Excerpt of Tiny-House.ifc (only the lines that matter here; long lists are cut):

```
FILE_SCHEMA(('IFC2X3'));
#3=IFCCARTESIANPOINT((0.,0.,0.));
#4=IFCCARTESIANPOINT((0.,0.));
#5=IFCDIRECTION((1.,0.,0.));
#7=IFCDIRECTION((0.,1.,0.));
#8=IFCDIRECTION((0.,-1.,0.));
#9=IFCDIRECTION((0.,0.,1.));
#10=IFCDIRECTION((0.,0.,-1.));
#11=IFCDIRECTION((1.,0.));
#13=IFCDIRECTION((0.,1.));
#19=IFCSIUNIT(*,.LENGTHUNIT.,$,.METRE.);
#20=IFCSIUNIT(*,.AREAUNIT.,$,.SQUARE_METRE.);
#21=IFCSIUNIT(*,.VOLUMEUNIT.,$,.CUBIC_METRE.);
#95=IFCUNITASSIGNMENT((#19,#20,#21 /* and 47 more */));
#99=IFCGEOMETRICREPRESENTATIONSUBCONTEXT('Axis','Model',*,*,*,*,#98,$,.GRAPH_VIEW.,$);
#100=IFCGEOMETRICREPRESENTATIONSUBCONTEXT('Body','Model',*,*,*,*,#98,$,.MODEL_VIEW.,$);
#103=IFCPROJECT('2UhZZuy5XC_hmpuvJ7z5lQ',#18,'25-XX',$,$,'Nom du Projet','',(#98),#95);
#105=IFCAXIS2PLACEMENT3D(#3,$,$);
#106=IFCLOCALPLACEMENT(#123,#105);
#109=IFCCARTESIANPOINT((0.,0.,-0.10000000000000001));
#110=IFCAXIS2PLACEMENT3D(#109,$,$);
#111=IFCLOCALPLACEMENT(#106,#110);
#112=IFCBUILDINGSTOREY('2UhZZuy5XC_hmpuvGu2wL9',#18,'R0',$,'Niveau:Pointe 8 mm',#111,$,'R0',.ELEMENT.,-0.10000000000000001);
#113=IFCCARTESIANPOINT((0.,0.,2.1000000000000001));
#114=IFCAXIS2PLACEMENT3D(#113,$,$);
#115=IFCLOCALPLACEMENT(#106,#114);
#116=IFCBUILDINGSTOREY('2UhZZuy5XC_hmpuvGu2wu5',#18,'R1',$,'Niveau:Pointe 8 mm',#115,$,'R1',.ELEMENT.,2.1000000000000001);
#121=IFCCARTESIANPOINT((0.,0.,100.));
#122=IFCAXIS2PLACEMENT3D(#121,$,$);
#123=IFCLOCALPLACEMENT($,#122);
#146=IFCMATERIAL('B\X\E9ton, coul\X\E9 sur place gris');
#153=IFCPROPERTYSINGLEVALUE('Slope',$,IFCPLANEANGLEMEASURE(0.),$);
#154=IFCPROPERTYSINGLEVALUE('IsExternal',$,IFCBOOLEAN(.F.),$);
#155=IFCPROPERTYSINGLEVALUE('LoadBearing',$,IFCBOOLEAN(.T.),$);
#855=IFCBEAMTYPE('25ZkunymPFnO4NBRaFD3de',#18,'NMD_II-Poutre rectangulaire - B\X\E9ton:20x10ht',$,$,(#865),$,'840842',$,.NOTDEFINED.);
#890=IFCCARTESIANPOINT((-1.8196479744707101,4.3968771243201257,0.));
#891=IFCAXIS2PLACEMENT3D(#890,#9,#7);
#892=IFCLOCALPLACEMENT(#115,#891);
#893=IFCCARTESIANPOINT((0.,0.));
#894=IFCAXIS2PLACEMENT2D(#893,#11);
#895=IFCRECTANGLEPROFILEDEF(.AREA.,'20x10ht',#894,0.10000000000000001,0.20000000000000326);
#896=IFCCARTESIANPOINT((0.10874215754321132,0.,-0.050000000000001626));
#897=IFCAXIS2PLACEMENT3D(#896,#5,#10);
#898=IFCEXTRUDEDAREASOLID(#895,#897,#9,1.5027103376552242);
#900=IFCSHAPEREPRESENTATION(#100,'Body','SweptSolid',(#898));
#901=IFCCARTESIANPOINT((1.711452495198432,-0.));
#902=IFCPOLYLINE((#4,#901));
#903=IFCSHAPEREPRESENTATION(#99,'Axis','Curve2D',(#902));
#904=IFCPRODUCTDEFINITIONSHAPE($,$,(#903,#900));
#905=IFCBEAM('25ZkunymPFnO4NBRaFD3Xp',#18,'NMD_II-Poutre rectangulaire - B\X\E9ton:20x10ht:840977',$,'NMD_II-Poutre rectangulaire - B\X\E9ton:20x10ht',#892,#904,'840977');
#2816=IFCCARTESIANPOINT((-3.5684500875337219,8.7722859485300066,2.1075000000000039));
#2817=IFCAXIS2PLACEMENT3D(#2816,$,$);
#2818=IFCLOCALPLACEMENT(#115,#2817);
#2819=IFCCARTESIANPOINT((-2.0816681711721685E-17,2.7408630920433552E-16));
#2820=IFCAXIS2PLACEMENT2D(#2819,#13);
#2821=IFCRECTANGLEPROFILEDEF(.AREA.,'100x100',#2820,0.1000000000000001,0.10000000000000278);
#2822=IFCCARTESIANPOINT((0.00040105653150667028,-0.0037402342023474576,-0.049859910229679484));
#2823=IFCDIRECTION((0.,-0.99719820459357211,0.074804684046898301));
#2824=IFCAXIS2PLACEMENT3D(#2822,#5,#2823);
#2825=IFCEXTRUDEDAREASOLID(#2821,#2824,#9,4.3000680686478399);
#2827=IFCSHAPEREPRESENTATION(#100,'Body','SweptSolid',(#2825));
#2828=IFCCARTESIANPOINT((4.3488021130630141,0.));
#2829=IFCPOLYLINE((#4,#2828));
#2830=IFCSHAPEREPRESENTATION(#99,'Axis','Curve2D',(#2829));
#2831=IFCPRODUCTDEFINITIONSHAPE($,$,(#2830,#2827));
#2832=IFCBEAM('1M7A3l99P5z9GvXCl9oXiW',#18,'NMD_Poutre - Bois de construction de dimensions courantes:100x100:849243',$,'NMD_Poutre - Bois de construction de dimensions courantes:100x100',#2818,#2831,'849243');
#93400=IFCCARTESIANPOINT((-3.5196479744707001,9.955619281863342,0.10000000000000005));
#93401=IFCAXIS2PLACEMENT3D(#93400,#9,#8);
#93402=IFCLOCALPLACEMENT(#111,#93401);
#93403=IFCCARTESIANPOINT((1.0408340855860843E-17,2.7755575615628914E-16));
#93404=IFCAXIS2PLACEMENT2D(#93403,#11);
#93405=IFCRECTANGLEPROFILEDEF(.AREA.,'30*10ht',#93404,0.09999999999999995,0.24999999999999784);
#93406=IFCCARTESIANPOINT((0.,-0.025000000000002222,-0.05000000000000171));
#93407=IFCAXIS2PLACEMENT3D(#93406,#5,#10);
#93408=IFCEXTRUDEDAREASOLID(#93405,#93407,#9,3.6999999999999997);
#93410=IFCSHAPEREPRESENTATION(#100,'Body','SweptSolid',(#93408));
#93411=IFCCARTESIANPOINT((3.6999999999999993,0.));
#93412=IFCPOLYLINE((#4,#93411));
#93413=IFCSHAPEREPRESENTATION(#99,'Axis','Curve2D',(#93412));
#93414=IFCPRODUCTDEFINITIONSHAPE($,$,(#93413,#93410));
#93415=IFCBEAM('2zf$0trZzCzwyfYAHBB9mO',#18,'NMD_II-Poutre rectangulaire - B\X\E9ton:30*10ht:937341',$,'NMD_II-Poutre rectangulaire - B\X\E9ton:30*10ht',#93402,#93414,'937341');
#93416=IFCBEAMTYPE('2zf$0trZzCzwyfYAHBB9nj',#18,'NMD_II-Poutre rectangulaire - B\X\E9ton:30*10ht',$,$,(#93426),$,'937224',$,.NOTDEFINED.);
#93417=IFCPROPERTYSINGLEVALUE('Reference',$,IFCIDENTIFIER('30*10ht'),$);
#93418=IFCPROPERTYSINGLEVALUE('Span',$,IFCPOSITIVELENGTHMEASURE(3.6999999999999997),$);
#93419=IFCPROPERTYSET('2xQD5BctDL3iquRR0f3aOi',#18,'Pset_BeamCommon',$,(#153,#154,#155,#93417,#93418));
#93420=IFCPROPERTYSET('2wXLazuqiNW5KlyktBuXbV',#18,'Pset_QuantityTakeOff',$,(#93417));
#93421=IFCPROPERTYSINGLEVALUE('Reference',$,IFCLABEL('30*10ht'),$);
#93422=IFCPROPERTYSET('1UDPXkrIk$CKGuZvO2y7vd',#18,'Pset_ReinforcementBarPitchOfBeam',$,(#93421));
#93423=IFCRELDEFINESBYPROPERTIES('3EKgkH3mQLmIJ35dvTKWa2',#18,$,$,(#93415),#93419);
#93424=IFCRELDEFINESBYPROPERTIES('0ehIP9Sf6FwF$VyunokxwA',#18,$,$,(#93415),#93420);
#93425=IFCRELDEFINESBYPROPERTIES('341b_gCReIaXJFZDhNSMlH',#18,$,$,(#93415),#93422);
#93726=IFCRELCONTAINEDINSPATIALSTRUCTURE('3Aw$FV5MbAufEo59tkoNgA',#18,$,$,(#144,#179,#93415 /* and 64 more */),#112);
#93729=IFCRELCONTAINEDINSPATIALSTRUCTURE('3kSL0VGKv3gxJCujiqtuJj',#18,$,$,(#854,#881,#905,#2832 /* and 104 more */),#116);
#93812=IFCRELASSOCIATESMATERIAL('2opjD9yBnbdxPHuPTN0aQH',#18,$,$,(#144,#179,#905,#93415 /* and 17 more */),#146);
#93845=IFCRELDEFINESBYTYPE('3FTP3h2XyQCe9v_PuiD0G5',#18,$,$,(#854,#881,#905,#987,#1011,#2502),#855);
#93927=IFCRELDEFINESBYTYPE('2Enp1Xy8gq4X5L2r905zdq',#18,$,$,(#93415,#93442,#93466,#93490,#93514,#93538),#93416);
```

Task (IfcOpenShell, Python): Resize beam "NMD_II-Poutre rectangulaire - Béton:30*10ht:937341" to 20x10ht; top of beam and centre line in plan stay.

```python
import ifcopenshell
import ifcopenshell.api.pset
import ifcopenshell.api.type
import ifcopenshell.util.element
import ifcopenshell.util.representation

model = ifcopenshell.open("Tiny-House.ifc")

member = model.by_guid("2zf$0trZzCzwyfYAHBB9mO")
source = next(p for p in model.by_type("IfcRectangleProfileDef") if p.ProfileName == "20x10ht")

body = ifcopenshell.util.representation.get_representation(member, "Model", "Body")
solid = body.Items[0]
old_profile = solid.SweptArea

# Copy the section's sizes but keep this member's own profile position.
profile = ifcopenshell.util.element.copy(model, source)
# Profiles are centred, so shift by half the change in depth to hold the top.
shift = (old_profile.XDim - profile.XDim) / 2
x, y = old_profile.Position.Location.Coordinates
up = (-1.0, 0.0)  # upwards, in the solid's own plane
location = model.createIfcCartesianPoint((x + up[0] * shift, y + up[1] * shift))
profile.Position = model.createIfcAxis2Placement2D(location, old_profile.Position.RefDirection)
solid.SweptArea = profile
if not model.get_total_inverses(old_profile):
    ifcopenshell.util.element.remove_deep2(model, old_profile)

new_type = model.by_id(855)
ifcopenshell.api.type.assign_type(
    model, related_objects=[member], relating_type=new_type, should_map_representations=False
)
member.Name = member.Name.replace("30*10ht", "20x10ht")
member.ObjectType = "NMD_II-Poutre rectangulaire - Béton:20x10ht"
pset = model.by_id(ifcopenshell.util.element.get_pset(member, "Pset_BeamCommon", should_inherit=False)["id"])
ifcopenshell.api.pset.edit_pset(model, pset=pset, properties={"Reference": "20x10ht"})
pset = model.by_id(ifcopenshell.util.element.get_pset(member, "Pset_QuantityTakeOff", should_inherit=False)["id"])
ifcopenshell.api.pset.edit_pset(model, pset=pset, properties={"Reference": "20x10ht"})
pset = model.by_id(ifcopenshell.util.element.get_pset(member, "Pset_ReinforcementBarPitchOfBeam", should_inherit=False)["id"])
ifcopenshell.api.pset.edit_pset(model, pset=pset, properties={"Reference": "20x10ht"})

print(solid.SweptArea)

model.write("Tiny-House_rev.ifc")
```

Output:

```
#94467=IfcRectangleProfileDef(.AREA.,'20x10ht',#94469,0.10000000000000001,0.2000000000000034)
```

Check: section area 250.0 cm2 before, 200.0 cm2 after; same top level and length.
